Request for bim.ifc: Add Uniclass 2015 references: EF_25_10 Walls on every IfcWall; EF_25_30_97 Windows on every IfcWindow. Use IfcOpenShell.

First a look at what the model holds.

```python
import ifcopenshell

model = ifcopenshell.open("bim.ifc")
print(model.schema)
print("classifications:", [c.Name for c in model.by_type("IfcClassification")])
for ifc_class in ("IfcDoor", "IfcRoof", "IfcStair", "IfcWall", "IfcWindow"):
    print(ifc_class, len(model.by_type(ifc_class)))
```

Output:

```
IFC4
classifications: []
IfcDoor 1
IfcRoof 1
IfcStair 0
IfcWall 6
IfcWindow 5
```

```python
import ifcopenshell
import ifcopenshell.api.classification

model = ifcopenshell.open("bim.ifc")

system = ifcopenshell.api.classification.add_classification(model, classification="Uniclass 2015")

codes = {
    "IfcWall": ("EF_25_10", "Walls"),
    "IfcWindow": ("EF_25_30_97", "Windows"),
}
for ifc_class, (code, name) in codes.items():
    products = model.by_type(ifc_class)
    ifcopenshell.api.classification.add_reference(
        model, products=products, classification=system, identification=code, name=name
    )
    print(code, len(products))

model.write("bim_rev.ifc")
```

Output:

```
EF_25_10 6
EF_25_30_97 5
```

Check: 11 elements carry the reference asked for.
